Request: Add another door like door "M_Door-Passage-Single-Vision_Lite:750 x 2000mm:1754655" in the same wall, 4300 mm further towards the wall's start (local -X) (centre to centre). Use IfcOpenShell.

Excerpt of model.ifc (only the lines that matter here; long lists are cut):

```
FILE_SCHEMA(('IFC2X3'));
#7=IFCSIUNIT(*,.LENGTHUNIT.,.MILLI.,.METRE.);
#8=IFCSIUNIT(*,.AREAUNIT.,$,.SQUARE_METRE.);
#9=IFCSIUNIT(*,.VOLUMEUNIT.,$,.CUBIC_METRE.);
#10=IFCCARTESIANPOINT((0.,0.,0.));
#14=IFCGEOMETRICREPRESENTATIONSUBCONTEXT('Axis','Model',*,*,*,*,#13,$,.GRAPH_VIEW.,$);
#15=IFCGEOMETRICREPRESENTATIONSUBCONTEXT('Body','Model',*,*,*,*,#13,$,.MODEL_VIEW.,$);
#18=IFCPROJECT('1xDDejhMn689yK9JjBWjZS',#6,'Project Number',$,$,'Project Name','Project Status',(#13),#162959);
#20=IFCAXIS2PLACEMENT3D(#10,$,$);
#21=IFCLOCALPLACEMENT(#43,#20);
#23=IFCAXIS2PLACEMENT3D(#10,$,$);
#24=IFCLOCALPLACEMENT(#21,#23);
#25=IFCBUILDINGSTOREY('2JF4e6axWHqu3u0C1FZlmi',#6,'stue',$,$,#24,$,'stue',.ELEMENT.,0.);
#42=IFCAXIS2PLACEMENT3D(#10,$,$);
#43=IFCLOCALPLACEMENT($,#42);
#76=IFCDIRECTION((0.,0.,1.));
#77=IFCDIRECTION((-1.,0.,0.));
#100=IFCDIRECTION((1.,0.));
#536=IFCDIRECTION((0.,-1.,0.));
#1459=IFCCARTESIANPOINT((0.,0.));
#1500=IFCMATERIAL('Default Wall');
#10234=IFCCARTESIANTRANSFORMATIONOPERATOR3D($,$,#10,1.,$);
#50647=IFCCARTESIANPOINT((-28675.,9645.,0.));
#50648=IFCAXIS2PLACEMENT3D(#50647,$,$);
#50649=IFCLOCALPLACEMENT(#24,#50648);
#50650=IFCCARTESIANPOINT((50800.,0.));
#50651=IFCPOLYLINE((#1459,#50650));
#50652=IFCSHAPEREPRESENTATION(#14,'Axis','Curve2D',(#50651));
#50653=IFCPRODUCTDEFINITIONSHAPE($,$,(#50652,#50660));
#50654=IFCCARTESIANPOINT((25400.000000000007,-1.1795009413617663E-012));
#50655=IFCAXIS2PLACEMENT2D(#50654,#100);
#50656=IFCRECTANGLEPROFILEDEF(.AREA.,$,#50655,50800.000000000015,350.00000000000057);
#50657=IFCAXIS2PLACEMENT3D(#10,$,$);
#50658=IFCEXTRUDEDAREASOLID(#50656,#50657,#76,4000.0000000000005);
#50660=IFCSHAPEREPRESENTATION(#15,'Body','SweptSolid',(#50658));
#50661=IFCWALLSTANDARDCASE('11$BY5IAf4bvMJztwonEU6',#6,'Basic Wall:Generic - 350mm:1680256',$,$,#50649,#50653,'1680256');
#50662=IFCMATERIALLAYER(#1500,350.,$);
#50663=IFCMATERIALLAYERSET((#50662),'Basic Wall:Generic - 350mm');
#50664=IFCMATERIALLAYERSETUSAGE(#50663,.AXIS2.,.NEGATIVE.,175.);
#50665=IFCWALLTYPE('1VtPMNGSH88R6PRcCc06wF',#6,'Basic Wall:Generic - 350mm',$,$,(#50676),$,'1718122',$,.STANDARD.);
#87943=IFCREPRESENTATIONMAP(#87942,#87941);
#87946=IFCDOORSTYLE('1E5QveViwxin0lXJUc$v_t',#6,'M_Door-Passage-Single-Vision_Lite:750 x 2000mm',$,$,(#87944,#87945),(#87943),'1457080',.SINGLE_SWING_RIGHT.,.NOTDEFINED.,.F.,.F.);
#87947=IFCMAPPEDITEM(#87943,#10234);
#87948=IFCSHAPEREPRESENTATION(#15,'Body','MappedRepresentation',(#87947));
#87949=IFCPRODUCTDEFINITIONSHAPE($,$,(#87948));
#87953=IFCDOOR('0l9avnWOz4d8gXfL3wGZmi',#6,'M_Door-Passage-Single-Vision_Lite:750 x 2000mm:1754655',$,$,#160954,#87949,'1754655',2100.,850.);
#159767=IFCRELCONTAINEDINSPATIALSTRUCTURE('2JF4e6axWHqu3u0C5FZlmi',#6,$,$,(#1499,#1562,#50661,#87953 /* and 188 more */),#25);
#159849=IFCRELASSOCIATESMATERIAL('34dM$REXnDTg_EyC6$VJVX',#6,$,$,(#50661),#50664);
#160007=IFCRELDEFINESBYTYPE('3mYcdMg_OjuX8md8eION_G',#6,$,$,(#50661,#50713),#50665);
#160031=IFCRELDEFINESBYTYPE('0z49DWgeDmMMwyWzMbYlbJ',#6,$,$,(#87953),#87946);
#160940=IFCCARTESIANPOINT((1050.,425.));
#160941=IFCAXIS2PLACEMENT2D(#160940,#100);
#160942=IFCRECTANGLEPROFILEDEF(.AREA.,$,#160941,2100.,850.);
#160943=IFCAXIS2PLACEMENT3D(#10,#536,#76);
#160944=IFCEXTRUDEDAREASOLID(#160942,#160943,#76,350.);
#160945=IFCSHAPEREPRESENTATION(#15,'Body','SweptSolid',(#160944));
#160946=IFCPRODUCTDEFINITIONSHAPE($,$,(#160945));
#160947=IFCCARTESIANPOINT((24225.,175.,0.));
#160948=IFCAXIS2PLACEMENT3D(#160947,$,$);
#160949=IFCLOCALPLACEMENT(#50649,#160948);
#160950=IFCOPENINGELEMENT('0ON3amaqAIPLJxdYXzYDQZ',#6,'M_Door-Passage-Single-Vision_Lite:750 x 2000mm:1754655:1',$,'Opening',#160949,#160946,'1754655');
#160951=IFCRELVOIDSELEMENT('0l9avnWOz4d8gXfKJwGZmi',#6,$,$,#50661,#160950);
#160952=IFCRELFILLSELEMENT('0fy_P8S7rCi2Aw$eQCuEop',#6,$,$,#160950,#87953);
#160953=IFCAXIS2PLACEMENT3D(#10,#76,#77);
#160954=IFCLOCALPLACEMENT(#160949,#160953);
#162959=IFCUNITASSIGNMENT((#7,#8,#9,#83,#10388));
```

```python
import ifcopenshell
import ifcopenshell.api.feature
import ifcopenshell.api.geometry
import ifcopenshell.api.root
import ifcopenshell.geom
import ifcopenshell.util.element
import ifcopenshell.util.placement
import ifcopenshell.util.shape
import ifcopenshell.util.unit

model = ifcopenshell.open("model.ifc")
unit_scale = ifcopenshell.util.unit.calculate_unit_scale(model)
settings = ifcopenshell.geom.settings()


def volume(element):
    """Net volume in cubic metres, openings subtracted."""
    shape = ifcopenshell.geom.create_shape(settings, element)
    return ifcopenshell.util.shape.get_volume(shape.geometry)


def reuse_history(source, copy):
    """copy_class also copies each property set's owner history, people and application; keep the originals."""
    for rel in copy.IsDefinedBy:
        if rel.is_a("IfcRelDefinesByProperties") and (history := rel.RelatingPropertyDefinition.OwnerHistory):
            rel.RelatingPropertyDefinition.OwnerHistory = source.OwnerHistory
            ifcopenshell.util.element.remove_deep2(model, history)


door = model.by_guid("0l9avnWOz4d8gXfL3wGZmi")
opening = door.FillsVoids[0].RelatingOpeningElement
wall = opening.VoidsElements[0].RelatingBuildingElement
before = volume(wall)
shift = ifcopenshell.util.placement.get_local_placement(wall.ObjectPlacement)[:3, 0] * -4.3 / unit_scale

# copy_class copies the void relationship, type, container and properties, but no geometry.
new_opening = ifcopenshell.api.root.copy_class(model, product=opening)
new_opening.Representation = ifcopenshell.util.element.copy_deep(
    model, opening.Representation, exclude=["IfcGeometricRepresentationContext", "IfcRepresentationMap"]
)
new_opening.Name = "M_Door-Passage-Single-Vision_Lite:750 x 2000mm"
new_opening.Tag = None
new_door = ifcopenshell.api.root.copy_class(model, product=door)
new_door.Representation = ifcopenshell.util.element.copy_deep(
    model, door.Representation, exclude=["IfcGeometricRepresentationContext", "IfcRepresentationMap"]
)
new_door.Name = "M_Door-Passage-Single-Vision_Lite:750 x 2000mm"
new_door.Tag = None
reuse_history(door, new_door)
fills = ifcopenshell.api.feature.add_filling(model, opening=new_opening, element=new_door)
fills.OwnerHistory = new_door.OwnerHistory  # required in IFC2X3

for old, new in ((opening, new_opening), (door, new_door)):
    matrix = ifcopenshell.util.placement.get_local_placement(old.ObjectPlacement)
    matrix[:3, 3] += shift
    ifcopenshell.api.geometry.edit_object_placement(model, product=new, matrix=matrix, is_si=False)

after = volume(wall)

print(f"wall volume {before:.3f} -> {after:.3f} m3")

model.write("model_rev.ifc")
```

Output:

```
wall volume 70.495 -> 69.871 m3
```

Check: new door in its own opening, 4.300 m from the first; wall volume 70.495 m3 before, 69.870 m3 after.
